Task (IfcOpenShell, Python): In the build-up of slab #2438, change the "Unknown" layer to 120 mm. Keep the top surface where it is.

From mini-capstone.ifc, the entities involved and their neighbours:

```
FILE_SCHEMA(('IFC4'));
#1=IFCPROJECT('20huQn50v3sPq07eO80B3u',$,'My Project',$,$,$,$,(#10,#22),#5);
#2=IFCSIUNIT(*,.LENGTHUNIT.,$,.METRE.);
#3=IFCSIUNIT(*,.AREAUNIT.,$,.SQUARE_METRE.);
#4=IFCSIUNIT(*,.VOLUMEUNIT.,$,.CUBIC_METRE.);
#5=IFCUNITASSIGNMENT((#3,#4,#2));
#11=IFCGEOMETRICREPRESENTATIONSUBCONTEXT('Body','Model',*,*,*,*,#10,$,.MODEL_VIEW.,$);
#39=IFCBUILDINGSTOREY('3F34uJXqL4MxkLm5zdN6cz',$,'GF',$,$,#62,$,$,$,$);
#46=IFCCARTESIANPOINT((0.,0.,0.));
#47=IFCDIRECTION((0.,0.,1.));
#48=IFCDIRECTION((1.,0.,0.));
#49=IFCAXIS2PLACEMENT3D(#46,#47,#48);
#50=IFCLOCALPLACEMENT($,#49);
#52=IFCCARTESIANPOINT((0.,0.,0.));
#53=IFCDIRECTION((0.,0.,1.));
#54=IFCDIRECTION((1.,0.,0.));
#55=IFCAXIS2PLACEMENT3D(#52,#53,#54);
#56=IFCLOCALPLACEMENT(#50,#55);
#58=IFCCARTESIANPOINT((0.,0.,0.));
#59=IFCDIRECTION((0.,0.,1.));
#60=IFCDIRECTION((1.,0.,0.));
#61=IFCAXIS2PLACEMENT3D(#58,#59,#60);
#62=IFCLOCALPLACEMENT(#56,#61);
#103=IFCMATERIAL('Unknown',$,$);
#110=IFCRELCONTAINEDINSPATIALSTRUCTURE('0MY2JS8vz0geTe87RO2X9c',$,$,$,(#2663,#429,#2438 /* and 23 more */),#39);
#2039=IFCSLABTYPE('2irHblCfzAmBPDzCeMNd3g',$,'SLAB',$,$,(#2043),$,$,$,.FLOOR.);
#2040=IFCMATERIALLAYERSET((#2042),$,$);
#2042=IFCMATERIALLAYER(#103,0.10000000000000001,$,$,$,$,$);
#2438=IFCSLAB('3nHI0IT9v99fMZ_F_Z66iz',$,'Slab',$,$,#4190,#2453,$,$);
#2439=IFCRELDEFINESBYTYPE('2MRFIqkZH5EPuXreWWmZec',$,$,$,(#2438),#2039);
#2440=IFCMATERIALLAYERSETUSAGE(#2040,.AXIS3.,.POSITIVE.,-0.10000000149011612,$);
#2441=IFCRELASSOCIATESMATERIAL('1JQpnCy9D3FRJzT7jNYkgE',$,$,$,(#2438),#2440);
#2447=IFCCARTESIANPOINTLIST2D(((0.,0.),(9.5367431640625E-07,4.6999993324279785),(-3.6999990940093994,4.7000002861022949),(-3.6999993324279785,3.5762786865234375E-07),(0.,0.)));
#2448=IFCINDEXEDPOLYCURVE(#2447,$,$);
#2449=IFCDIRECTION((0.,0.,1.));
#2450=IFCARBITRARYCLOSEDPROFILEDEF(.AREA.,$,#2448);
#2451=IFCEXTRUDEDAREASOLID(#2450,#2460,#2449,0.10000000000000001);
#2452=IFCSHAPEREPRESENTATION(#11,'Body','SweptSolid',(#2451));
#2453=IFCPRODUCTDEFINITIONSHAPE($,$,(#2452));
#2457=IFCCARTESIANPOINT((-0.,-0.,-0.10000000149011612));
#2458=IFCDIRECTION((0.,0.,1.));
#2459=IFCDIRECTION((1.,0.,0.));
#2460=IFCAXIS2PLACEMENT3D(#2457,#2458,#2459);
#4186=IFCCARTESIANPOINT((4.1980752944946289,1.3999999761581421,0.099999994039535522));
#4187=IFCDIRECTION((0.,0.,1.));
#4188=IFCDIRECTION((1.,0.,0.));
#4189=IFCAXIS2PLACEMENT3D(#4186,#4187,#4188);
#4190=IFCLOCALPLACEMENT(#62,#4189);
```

```python
import ifcopenshell
import ifcopenshell.util.element
import ifcopenshell.util.representation

model = ifcopenshell.open("mini-capstone.ifc")

layer_set = model.by_id(2040)
layer = next(l for l in layer_set.MaterialLayers if l.Material and l.Material.Name == "Unknown")
change = 0.12 - layer.LayerThickness
layer.LayerThickness += change

# Geometry does not follow the layer set by itself.
slabs = [e for e in ifcopenshell.util.element.get_elements_by_material(model, layer_set) if e.is_a("IfcSlab")]
for slab in sorted(slabs, key=lambda e: e.id()):
    body = ifcopenshell.util.representation.get_representation(slab, "Model", "Body")
    solid = body.Items[0]
    old_depth = solid.Depth
    solid.Depth += change
    # Extruded upwards: lower the start of the extrusion so the top stays.
    x, y, z = solid.Position.Location.Coordinates
    solid.Position.Location = model.createIfcCartesianPoint((x, y, z - change))
    print(slab.id(), f"{old_depth:g} -> {solid.Depth:g}")

# The layers are counted up from the underside, which has moved.
for usage in {ifcopenshell.util.element.get_material(slab) for slab in slabs}:
    usage.OffsetFromReferenceLine -= change

model.write("mini-capstone-out.ifc")
```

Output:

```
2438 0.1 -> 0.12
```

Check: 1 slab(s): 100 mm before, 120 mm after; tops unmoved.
